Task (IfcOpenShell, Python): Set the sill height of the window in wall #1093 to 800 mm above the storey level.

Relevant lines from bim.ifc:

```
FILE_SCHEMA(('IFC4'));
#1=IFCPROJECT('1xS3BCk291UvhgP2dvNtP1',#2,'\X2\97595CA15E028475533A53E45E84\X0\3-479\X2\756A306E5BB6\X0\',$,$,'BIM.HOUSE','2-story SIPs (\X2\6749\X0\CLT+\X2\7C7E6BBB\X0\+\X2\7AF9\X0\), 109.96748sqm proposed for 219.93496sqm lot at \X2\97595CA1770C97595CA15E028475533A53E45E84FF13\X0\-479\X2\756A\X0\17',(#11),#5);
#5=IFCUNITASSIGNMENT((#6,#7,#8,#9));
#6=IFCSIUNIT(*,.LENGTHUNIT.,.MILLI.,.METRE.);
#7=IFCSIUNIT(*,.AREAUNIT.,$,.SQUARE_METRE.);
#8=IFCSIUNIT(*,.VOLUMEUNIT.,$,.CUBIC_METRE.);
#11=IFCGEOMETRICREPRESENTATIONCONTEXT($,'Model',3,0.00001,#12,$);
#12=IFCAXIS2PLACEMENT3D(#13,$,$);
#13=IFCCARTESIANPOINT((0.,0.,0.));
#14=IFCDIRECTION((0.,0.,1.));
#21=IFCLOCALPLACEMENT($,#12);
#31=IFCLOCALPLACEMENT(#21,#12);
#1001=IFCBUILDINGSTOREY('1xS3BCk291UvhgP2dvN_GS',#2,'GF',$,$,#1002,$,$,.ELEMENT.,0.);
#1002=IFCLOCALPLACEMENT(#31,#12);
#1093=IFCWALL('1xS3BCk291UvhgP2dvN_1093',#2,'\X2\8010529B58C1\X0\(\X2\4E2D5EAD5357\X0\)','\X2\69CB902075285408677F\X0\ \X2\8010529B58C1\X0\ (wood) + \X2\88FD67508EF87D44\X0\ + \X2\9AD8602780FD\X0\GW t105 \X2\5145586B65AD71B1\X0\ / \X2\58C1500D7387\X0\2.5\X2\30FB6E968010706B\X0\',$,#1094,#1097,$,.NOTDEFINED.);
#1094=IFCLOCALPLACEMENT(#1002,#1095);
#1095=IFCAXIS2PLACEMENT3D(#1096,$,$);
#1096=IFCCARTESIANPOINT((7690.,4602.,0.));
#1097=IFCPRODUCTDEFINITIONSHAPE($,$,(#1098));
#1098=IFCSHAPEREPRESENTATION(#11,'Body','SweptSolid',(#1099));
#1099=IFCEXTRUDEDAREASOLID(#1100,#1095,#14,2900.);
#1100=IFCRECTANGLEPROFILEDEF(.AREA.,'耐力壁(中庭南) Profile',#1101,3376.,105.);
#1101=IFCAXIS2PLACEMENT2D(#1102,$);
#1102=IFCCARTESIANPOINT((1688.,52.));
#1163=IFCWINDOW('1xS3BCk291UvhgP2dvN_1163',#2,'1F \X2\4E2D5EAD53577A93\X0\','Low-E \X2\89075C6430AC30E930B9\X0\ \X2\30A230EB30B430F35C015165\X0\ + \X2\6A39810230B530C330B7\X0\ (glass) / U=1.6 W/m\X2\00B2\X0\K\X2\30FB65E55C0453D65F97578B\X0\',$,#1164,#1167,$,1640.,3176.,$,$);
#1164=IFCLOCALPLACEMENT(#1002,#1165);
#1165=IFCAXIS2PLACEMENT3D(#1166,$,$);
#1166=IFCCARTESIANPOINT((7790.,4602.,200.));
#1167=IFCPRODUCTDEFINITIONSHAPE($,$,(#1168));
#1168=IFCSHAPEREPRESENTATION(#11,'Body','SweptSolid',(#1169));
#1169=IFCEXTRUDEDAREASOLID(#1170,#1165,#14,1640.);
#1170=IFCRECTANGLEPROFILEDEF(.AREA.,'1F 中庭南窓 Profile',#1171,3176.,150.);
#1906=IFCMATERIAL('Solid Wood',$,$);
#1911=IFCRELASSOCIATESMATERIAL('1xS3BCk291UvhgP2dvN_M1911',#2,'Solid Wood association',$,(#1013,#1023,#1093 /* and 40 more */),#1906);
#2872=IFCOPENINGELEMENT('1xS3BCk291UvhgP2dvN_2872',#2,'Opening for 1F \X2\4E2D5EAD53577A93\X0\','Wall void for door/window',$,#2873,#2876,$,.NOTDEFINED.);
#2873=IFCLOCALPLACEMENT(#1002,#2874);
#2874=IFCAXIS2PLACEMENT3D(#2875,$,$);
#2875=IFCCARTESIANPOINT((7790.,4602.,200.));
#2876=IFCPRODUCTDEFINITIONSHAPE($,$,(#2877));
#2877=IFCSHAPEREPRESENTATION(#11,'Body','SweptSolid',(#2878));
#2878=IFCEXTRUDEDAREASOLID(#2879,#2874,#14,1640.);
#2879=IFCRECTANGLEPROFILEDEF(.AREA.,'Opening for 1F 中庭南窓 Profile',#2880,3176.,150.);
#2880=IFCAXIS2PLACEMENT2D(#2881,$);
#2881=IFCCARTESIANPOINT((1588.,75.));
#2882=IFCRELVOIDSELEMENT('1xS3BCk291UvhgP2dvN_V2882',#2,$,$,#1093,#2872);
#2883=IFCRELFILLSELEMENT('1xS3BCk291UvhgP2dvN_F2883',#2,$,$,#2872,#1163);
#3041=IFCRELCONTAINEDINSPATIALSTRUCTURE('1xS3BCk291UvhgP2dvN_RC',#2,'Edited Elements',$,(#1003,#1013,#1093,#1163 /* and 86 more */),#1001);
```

```python
import numpy as np
import ifcopenshell
import ifcopenshell.api.geometry
import ifcopenshell.geom
import ifcopenshell.util.element
import ifcopenshell.util.placement
import ifcopenshell.util.shape
import ifcopenshell.util.unit

model = ifcopenshell.open("bim.ifc")
unit_scale = ifcopenshell.util.unit.calculate_unit_scale(model)

window = model.by_guid("1xS3BCk291UvhgP2dvN_1163")
opening = window.FillsVoids[0].RelatingOpeningElement
storey = ifcopenshell.util.element.get_container(window, ifc_class="IfcBuildingStorey")
level = ifcopenshell.util.placement.get_local_placement(storey.ObjectPlacement)[2, 3]

# The opening's origin need not be at the sill, so measure its lowest point.
shape = ifcopenshell.geom.create_shape(ifcopenshell.geom.settings(), opening)
bottom = ifcopenshell.util.shape.get_shape_bottom_elevation(shape, shape.geometry) / unit_scale
dz = level + 800.0 - bottom

shift = np.array([0.0, 0.0, dz])
# The window is not placed relative to its opening, so move both.
for product in (opening, window):
    matrix = ifcopenshell.util.placement.get_local_placement(product.ObjectPlacement)
    matrix[:3, 3] += shift
    ifcopenshell.api.geometry.edit_object_placement(model, product=product, matrix=matrix, is_si=False)

print(f"moved by {dz * unit_scale:+.3f} m")

model.write("bim_updated.ifc")
```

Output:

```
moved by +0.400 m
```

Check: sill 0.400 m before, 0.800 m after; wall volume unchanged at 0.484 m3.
